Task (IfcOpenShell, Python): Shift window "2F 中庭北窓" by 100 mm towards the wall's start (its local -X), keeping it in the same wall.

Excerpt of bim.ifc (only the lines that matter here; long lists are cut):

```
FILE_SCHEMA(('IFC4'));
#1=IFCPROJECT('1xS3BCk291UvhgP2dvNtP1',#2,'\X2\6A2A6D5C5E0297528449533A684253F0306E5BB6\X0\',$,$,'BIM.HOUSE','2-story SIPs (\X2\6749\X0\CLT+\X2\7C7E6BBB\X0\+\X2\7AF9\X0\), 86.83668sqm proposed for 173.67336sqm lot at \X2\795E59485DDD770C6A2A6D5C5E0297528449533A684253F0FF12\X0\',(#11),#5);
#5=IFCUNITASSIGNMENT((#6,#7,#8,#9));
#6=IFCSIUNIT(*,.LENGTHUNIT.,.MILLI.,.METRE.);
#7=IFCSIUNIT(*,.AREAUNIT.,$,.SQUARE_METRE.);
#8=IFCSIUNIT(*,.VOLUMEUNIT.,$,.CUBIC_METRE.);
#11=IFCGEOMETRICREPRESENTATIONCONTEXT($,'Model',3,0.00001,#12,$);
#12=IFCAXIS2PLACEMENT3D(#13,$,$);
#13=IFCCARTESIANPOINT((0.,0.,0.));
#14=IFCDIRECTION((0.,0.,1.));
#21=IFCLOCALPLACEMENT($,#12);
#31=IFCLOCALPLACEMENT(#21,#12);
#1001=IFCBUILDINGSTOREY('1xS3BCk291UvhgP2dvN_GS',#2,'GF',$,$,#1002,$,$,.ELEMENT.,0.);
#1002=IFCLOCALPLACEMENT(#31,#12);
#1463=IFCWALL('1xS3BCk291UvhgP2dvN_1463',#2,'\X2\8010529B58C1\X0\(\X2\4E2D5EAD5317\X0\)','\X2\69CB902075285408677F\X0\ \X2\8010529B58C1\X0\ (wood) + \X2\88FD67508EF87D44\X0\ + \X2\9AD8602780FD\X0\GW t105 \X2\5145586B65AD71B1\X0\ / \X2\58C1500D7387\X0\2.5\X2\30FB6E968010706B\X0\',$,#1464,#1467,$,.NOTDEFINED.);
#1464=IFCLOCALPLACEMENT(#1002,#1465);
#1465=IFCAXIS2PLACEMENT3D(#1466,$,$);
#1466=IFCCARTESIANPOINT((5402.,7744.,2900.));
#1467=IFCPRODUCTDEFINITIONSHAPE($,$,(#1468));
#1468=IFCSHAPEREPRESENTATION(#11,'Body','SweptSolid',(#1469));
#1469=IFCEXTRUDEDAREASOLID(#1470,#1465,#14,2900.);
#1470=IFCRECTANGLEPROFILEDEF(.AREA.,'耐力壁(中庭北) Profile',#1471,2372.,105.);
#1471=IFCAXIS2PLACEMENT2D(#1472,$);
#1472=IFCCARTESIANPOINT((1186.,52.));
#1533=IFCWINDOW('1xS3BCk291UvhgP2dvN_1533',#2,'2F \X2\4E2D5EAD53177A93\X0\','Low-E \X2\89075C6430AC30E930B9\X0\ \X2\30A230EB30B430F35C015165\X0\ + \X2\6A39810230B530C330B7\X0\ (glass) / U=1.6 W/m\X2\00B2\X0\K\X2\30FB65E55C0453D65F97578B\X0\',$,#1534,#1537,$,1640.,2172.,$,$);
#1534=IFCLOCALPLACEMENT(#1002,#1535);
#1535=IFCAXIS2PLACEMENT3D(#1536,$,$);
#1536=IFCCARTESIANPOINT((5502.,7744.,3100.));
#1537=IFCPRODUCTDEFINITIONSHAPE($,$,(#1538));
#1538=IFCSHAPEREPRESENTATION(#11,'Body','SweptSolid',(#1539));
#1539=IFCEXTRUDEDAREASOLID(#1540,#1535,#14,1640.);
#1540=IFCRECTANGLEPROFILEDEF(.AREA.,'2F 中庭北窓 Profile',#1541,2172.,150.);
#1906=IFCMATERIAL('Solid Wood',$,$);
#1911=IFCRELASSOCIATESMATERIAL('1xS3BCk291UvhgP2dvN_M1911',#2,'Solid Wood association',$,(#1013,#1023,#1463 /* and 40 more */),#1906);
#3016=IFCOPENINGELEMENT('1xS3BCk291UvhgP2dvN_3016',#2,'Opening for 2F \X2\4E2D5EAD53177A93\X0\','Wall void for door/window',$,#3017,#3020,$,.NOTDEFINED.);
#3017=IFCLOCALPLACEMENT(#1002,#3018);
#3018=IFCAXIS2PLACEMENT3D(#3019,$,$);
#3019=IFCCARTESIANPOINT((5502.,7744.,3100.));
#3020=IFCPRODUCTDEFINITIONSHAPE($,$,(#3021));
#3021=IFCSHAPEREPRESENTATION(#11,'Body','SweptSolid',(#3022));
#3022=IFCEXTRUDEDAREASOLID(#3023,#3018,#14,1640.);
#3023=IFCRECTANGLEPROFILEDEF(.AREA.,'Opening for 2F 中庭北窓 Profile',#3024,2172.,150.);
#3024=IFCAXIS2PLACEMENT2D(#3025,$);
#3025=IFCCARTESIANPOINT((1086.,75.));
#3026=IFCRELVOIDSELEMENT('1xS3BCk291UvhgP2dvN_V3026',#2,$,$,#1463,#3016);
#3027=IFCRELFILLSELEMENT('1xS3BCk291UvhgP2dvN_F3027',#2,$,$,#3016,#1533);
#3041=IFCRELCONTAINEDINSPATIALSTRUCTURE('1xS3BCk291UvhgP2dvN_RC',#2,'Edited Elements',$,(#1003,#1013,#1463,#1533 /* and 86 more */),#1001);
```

```python
import ifcopenshell
import ifcopenshell.api.geometry
import ifcopenshell.util.placement
import ifcopenshell.util.unit

model = ifcopenshell.open("bim.ifc")
unit_scale = ifcopenshell.util.unit.calculate_unit_scale(model)

window = model.by_guid("1xS3BCk291UvhgP2dvN_1533")
opening = window.FillsVoids[0].RelatingOpeningElement
wall = opening.VoidsElements[0].RelatingBuildingElement

wall_matrix = ifcopenshell.util.placement.get_local_placement(wall.ObjectPlacement)
shift = wall_matrix[:3, 0] * -0.1 / unit_scale
before = ifcopenshell.util.placement.get_local_placement(window.ObjectPlacement)[:3, 3].copy()

# The window is not placed relative to its opening, so move both.
for product in (opening, window):
    matrix = ifcopenshell.util.placement.get_local_placement(product.ObjectPlacement)
    matrix[:3, 3] += shift
    ifcopenshell.api.geometry.edit_object_placement(model, product=product, matrix=matrix, is_si=False)

after = ifcopenshell.util.placement.get_local_placement(window.ObjectPlacement)[:3, 3]
print("window moved by", (after - before).round(3) + 0.0)

model.write("bim_updated.ifc")
```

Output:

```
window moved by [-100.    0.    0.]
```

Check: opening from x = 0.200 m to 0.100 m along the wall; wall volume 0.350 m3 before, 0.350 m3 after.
